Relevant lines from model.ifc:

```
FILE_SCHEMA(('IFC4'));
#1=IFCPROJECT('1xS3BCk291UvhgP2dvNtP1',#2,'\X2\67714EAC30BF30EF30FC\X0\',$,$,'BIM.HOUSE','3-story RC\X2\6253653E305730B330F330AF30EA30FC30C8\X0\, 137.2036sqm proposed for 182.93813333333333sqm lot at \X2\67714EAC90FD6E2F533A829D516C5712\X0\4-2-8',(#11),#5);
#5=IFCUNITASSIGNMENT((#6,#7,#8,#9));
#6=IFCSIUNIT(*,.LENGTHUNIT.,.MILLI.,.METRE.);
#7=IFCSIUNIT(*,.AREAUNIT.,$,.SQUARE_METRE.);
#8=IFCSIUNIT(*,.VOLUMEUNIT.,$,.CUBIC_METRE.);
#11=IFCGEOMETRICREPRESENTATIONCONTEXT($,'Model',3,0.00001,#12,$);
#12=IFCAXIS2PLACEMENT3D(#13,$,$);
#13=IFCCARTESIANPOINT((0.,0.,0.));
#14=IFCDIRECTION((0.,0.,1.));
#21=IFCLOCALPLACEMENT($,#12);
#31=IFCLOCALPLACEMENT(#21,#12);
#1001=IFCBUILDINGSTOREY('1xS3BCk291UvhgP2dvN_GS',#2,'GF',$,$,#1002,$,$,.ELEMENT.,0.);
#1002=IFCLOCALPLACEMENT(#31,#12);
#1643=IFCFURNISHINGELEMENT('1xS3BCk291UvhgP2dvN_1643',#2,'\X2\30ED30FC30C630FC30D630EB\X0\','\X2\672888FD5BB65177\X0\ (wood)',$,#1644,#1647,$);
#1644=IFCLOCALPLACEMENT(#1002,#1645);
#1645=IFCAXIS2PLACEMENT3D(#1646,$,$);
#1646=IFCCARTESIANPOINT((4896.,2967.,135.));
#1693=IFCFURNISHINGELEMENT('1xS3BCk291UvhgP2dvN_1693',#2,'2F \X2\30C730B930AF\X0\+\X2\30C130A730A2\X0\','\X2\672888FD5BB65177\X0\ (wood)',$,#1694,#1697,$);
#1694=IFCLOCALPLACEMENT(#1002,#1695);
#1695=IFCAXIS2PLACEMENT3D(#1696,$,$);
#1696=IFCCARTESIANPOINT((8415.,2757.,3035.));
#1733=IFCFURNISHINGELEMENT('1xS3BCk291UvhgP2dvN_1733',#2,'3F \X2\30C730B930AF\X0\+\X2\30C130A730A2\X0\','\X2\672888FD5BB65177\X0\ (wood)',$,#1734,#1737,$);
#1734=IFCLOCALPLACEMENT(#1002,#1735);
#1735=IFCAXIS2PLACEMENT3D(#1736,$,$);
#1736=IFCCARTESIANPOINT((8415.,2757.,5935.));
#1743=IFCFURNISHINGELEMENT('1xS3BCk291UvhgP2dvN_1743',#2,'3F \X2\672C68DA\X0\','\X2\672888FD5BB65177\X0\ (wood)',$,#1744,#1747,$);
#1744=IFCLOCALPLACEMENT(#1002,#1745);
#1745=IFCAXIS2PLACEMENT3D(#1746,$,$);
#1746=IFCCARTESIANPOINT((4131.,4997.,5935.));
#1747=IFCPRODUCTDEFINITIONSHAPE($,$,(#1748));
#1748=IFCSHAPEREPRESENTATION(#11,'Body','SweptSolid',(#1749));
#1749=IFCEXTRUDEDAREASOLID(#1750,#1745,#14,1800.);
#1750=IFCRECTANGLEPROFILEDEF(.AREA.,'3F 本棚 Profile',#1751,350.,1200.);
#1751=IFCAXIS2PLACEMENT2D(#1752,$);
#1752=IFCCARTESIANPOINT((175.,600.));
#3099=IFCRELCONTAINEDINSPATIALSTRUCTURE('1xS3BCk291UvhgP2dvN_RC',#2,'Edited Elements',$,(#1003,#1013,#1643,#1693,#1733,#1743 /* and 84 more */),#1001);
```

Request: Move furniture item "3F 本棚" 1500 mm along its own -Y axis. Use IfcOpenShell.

```python
import ifcopenshell
import ifcopenshell.api.geometry
import ifcopenshell.util.placement
import ifcopenshell.util.unit

model = ifcopenshell.open("model.ifc")
unit_scale = ifcopenshell.util.unit.calculate_unit_scale(model)

item = model.by_guid("1xS3BCk291UvhgP2dvN_1743")
matrix = ifcopenshell.util.placement.get_local_placement(item.ObjectPlacement)
matrix[:3, 3] -= matrix[:3, 1] * 1.5 / unit_scale
ifcopenshell.api.geometry.edit_object_placement(model, product=item, matrix=matrix, is_si=False)

print(ifcopenshell.util.placement.get_local_placement(item.ObjectPlacement).round(3) + 0.0)

model.write("model_rev.ifc")
```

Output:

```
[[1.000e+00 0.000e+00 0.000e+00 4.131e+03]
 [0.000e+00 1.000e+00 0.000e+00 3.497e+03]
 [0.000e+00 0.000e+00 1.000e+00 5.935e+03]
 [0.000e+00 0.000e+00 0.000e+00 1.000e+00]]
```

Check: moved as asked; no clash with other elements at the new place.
